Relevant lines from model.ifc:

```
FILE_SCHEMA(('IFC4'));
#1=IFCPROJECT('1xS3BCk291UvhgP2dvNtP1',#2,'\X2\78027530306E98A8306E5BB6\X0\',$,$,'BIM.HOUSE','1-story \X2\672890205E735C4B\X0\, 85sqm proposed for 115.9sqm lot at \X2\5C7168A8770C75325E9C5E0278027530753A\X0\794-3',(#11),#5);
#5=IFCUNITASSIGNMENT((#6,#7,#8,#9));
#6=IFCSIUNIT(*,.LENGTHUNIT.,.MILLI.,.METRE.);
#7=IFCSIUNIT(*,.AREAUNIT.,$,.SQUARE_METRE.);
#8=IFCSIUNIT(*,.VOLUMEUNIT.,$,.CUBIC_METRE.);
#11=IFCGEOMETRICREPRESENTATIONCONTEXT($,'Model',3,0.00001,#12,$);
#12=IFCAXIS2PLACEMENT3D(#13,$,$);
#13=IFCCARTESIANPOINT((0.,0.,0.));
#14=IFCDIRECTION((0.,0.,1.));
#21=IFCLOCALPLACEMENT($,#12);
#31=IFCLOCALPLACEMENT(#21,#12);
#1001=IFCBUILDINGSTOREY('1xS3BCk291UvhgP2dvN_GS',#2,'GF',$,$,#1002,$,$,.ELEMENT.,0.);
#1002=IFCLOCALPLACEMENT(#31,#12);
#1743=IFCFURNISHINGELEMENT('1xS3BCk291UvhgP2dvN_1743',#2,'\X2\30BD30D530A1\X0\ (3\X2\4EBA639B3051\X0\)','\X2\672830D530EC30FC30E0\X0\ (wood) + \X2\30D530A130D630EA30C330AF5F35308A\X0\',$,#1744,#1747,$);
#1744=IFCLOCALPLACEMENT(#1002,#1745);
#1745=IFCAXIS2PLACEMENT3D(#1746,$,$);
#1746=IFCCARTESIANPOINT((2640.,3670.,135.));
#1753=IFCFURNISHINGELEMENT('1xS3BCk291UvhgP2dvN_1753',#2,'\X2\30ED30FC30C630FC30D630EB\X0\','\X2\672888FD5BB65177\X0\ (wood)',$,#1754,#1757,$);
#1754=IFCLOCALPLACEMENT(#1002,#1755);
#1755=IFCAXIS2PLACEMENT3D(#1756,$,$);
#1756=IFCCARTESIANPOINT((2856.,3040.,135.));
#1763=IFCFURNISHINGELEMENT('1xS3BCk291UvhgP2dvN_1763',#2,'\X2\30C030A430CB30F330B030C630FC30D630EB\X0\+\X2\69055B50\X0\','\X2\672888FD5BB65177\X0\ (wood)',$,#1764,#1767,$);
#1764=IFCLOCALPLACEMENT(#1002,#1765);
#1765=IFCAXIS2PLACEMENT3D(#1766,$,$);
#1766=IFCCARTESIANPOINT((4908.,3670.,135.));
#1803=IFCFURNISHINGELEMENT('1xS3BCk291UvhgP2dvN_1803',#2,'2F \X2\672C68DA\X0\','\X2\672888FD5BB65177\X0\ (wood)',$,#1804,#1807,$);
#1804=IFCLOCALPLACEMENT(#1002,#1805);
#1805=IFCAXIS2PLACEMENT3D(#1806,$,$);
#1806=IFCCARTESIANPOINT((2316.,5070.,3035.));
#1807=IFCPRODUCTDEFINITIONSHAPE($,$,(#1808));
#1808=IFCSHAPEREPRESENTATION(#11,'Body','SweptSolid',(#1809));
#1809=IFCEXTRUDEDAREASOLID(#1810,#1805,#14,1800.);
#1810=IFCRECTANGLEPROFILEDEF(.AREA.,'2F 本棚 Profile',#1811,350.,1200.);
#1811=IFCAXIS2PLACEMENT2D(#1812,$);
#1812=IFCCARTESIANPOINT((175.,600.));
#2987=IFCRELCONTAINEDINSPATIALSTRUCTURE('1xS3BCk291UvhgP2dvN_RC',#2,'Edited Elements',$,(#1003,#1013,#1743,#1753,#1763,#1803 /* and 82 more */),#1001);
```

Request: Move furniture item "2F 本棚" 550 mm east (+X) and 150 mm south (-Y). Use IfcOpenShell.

```python
import ifcopenshell
import ifcopenshell.api.geometry
import ifcopenshell.util.placement

model = ifcopenshell.open("model.ifc")

item = model.by_id(1803)
matrix = ifcopenshell.util.placement.get_local_placement(item.ObjectPlacement)
matrix[0, 3] += 550.0
matrix[1, 3] -= 150.0
ifcopenshell.api.geometry.edit_object_placement(model, product=item, matrix=matrix, is_si=False)

print(ifcopenshell.util.placement.get_local_placement(item.ObjectPlacement).round(3) + 0.0)

model.write("model_edited.ifc")
```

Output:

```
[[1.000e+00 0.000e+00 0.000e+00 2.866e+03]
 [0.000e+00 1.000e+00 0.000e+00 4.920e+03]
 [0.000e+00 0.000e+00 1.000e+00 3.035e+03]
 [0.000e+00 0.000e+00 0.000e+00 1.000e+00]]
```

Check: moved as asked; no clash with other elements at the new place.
